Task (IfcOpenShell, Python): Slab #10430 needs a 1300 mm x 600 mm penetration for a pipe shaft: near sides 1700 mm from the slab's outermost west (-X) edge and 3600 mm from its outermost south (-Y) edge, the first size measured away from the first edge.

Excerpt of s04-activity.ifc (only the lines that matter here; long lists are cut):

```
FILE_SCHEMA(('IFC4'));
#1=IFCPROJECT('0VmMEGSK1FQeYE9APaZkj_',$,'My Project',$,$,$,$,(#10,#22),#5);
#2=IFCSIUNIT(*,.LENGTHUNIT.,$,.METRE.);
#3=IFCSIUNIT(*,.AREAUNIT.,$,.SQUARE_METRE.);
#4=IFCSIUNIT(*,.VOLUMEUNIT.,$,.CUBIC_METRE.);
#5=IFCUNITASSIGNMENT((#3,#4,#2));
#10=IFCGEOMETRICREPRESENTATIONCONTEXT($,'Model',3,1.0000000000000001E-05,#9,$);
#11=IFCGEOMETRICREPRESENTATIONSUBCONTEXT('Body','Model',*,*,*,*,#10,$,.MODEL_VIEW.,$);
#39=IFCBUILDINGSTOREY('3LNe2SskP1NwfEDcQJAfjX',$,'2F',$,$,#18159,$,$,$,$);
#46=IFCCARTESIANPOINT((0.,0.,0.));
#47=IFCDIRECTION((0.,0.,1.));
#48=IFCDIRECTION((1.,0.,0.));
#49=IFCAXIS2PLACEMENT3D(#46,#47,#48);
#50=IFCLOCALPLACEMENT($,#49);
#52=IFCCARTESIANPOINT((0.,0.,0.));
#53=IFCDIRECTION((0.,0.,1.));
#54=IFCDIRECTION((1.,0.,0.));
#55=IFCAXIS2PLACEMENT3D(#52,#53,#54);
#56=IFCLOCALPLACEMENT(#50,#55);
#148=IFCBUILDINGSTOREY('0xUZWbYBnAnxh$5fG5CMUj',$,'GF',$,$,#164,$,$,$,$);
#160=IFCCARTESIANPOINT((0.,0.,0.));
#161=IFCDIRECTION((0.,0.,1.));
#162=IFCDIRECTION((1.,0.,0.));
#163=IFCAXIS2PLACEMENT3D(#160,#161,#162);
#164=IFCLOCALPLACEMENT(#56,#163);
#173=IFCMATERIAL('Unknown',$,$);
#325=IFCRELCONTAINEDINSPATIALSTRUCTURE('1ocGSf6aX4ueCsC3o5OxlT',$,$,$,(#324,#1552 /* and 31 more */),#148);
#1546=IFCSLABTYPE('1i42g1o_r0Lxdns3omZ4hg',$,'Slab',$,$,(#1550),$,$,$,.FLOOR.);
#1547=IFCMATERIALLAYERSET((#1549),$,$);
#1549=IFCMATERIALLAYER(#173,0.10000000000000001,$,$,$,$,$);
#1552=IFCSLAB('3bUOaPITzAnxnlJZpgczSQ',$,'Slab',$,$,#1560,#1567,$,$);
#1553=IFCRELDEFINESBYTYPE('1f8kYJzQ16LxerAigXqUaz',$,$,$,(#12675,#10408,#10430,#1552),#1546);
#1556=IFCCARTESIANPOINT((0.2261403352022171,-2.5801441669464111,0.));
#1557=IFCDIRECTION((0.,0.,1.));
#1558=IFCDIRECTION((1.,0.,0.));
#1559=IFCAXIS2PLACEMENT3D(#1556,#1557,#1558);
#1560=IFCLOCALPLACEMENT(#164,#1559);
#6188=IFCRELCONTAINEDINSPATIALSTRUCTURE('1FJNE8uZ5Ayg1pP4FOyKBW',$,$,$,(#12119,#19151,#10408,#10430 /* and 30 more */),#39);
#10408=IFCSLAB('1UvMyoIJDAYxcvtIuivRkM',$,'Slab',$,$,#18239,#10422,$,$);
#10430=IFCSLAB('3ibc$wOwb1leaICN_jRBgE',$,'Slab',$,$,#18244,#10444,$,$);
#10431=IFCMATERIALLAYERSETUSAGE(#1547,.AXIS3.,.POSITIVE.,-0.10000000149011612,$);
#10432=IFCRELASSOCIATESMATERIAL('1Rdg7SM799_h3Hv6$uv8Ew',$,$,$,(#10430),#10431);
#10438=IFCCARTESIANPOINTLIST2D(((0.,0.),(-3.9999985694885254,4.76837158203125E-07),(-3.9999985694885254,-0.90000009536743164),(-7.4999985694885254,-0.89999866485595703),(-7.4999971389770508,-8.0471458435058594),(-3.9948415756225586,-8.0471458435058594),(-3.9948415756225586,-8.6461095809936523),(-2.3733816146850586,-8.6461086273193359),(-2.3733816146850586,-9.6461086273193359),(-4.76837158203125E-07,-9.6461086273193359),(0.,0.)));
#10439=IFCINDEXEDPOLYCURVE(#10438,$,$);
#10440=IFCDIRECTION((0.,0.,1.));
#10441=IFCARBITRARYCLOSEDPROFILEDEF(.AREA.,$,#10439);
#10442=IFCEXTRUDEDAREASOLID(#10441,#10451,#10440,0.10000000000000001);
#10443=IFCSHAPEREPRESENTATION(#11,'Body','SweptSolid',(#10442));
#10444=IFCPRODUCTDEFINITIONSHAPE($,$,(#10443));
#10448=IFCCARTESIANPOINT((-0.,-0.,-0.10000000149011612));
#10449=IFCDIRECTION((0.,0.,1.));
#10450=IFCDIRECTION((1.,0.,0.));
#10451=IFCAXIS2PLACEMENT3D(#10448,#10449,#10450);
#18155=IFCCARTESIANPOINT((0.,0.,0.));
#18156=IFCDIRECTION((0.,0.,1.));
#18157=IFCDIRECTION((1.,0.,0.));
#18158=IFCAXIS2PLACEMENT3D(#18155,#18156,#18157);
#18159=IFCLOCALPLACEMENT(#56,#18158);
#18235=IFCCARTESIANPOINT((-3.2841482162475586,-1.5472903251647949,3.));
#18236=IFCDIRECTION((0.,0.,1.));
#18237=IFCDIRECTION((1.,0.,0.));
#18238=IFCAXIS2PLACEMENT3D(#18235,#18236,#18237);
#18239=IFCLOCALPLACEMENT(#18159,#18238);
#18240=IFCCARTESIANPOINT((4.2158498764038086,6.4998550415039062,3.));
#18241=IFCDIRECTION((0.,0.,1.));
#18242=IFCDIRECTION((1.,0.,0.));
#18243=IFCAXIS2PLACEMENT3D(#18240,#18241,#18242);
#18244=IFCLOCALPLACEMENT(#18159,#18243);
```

```python
import numpy as np
import ifcopenshell
import ifcopenshell.api.feature
import ifcopenshell.api.geometry
import ifcopenshell.api.root
import ifcopenshell.geom
import ifcopenshell.util.placement
import ifcopenshell.util.representation
import ifcopenshell.util.shape
import ifcopenshell.util.unit

model = ifcopenshell.open("s04-activity.ifc")
unit_scale = ifcopenshell.util.unit.calculate_unit_scale(model)
settings = ifcopenshell.geom.settings()


def volume(element):
    """Net volume in cubic metres, openings subtracted."""
    shape = ifcopenshell.geom.create_shape(settings, element)
    return ifcopenshell.util.shape.get_volume(shape.geometry)


slab = model.by_id(10430)
before = volume(slab)

# Extent in the slab's own axes, in metres. The edges named are its -X and -Y sides.
slab_shape = ifcopenshell.geom.create_shape(settings, slab)
vertices = ifcopenshell.util.shape.get_vertices(slab_shape.geometry)
x_min, y_min, bottom = vertices.min(axis=0)
top = vertices[:, 2].max()

opening = ifcopenshell.api.root.create_entity(model, ifc_class="IfcOpeningElement", name="Pipe shaft opening", predefined_type="OPENING")
context = ifcopenshell.util.representation.get_context(model, "Model", "Body", "MODEL_VIEW")
width, depth = 1.3, 0.6
outline = [(0.0, 0.0), (width, 0.0), (width, depth), (0.0, depth), (0.0, 0.0)]
# Overshoot both faces by 50 mm so the cut is clean.
shape = ifcopenshell.api.geometry.add_slab_representation(
    model, context=context, depth=top - bottom + 0.1, polyline=outline
)
ifcopenshell.api.geometry.assign_representation(model, product=opening, representation=shape)

matrix = ifcopenshell.util.placement.get_local_placement(slab.ObjectPlacement)
matrix[:, 3] = matrix @ np.append(np.array([x_min + 1.7, y_min + 3.6, bottom - 0.05]) / unit_scale, 1.0)
ifcopenshell.api.geometry.edit_object_placement(model, product=opening, matrix=matrix, is_si=False)
ifcopenshell.api.feature.add_feature(model, feature=opening, element=slab)

after = volume(slab)

print(f"slab volume {before:.3f} -> {after:.3f} m3")

model.write("s04-activity_updated.ifc")
```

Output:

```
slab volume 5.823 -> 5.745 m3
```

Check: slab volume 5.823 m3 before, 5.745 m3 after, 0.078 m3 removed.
